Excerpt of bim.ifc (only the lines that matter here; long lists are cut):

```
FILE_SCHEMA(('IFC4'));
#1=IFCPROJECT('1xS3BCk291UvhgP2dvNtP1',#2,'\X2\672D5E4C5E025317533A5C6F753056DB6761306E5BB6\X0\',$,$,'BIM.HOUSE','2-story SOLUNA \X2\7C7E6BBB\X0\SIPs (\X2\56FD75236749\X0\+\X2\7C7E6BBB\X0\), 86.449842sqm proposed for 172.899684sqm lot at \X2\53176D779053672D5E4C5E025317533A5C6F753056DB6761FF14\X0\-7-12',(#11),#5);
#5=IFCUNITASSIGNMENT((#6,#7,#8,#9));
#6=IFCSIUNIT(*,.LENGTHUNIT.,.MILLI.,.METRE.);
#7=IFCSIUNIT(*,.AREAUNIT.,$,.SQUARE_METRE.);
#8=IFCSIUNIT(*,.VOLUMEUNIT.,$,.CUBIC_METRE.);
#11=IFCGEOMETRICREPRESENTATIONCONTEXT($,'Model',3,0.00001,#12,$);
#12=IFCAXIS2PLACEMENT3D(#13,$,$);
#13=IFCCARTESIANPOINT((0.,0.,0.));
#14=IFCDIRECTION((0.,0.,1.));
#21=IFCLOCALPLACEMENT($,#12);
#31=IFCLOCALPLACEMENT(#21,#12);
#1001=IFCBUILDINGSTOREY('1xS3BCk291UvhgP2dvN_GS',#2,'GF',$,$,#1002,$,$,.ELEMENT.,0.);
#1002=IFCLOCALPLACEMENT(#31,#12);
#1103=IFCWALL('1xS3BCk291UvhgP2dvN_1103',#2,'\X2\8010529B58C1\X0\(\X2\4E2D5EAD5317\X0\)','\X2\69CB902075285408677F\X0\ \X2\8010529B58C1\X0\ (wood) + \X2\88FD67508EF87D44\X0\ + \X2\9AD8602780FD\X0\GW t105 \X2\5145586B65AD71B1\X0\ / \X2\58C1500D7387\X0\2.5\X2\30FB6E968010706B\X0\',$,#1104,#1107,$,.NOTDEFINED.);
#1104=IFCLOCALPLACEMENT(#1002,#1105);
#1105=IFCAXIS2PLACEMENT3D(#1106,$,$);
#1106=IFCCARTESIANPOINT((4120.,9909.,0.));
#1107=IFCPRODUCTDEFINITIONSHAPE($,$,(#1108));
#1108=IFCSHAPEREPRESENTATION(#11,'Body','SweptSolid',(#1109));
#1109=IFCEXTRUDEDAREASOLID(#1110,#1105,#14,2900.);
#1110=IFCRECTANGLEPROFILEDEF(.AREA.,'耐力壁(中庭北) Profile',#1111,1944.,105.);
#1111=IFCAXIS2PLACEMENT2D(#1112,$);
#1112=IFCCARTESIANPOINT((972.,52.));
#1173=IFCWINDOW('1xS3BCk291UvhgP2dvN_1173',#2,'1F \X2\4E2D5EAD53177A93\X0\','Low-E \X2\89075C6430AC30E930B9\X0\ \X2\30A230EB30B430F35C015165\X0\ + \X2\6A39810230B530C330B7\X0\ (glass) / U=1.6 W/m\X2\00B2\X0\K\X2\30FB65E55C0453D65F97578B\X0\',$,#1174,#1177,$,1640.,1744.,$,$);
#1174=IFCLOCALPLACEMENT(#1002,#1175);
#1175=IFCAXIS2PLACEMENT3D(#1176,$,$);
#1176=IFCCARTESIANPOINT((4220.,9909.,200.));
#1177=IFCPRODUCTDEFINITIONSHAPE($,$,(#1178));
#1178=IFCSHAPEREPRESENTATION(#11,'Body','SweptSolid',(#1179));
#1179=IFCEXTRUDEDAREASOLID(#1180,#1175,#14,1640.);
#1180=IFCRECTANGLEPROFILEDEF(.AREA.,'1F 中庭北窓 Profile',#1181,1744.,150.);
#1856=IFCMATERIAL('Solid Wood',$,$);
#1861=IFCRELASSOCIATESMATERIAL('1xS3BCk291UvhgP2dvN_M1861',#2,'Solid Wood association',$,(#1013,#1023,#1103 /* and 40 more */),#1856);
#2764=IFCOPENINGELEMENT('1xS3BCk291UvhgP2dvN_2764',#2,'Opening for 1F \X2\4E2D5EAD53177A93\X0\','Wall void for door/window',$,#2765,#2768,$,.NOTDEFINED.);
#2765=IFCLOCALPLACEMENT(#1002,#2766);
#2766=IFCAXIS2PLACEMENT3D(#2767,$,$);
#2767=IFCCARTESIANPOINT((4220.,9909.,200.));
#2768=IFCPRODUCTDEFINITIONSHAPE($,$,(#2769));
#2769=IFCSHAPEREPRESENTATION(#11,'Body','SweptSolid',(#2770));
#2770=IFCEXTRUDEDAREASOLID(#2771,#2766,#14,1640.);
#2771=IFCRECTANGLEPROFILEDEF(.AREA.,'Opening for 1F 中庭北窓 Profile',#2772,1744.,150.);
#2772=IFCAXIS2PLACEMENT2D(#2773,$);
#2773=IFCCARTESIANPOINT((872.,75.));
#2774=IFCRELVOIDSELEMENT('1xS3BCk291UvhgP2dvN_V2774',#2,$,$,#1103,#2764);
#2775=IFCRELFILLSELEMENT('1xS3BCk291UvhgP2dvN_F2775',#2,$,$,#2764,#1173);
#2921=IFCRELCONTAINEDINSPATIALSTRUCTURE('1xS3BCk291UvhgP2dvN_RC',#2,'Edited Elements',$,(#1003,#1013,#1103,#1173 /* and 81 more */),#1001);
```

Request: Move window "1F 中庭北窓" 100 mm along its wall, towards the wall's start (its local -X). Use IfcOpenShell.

```python
import ifcopenshell
import ifcopenshell.api.geometry
import ifcopenshell.util.placement

model = ifcopenshell.open("bim.ifc")

window = model.by_id(1173)
opening = window.FillsVoids[0].RelatingOpeningElement
wall = opening.VoidsElements[0].RelatingBuildingElement

wall_matrix = ifcopenshell.util.placement.get_local_placement(wall.ObjectPlacement)
shift = wall_matrix[:3, 0] * -100.0
before = ifcopenshell.util.placement.get_local_placement(window.ObjectPlacement)[:3, 3].copy()

# The window is not placed relative to its opening, so move both.
for product in (opening, window):
    matrix = ifcopenshell.util.placement.get_local_placement(product.ObjectPlacement)
    matrix[:3, 3] += shift
    ifcopenshell.api.geometry.edit_object_placement(model, product=product, matrix=matrix, is_si=False)

after = ifcopenshell.util.placement.get_local_placement(window.ObjectPlacement)[:3, 3]
print("window moved by", (after - before).round(3) + 0.0)

model.write("bim_edited.ifc")
```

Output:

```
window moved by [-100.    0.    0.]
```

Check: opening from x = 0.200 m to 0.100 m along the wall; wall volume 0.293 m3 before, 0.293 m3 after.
